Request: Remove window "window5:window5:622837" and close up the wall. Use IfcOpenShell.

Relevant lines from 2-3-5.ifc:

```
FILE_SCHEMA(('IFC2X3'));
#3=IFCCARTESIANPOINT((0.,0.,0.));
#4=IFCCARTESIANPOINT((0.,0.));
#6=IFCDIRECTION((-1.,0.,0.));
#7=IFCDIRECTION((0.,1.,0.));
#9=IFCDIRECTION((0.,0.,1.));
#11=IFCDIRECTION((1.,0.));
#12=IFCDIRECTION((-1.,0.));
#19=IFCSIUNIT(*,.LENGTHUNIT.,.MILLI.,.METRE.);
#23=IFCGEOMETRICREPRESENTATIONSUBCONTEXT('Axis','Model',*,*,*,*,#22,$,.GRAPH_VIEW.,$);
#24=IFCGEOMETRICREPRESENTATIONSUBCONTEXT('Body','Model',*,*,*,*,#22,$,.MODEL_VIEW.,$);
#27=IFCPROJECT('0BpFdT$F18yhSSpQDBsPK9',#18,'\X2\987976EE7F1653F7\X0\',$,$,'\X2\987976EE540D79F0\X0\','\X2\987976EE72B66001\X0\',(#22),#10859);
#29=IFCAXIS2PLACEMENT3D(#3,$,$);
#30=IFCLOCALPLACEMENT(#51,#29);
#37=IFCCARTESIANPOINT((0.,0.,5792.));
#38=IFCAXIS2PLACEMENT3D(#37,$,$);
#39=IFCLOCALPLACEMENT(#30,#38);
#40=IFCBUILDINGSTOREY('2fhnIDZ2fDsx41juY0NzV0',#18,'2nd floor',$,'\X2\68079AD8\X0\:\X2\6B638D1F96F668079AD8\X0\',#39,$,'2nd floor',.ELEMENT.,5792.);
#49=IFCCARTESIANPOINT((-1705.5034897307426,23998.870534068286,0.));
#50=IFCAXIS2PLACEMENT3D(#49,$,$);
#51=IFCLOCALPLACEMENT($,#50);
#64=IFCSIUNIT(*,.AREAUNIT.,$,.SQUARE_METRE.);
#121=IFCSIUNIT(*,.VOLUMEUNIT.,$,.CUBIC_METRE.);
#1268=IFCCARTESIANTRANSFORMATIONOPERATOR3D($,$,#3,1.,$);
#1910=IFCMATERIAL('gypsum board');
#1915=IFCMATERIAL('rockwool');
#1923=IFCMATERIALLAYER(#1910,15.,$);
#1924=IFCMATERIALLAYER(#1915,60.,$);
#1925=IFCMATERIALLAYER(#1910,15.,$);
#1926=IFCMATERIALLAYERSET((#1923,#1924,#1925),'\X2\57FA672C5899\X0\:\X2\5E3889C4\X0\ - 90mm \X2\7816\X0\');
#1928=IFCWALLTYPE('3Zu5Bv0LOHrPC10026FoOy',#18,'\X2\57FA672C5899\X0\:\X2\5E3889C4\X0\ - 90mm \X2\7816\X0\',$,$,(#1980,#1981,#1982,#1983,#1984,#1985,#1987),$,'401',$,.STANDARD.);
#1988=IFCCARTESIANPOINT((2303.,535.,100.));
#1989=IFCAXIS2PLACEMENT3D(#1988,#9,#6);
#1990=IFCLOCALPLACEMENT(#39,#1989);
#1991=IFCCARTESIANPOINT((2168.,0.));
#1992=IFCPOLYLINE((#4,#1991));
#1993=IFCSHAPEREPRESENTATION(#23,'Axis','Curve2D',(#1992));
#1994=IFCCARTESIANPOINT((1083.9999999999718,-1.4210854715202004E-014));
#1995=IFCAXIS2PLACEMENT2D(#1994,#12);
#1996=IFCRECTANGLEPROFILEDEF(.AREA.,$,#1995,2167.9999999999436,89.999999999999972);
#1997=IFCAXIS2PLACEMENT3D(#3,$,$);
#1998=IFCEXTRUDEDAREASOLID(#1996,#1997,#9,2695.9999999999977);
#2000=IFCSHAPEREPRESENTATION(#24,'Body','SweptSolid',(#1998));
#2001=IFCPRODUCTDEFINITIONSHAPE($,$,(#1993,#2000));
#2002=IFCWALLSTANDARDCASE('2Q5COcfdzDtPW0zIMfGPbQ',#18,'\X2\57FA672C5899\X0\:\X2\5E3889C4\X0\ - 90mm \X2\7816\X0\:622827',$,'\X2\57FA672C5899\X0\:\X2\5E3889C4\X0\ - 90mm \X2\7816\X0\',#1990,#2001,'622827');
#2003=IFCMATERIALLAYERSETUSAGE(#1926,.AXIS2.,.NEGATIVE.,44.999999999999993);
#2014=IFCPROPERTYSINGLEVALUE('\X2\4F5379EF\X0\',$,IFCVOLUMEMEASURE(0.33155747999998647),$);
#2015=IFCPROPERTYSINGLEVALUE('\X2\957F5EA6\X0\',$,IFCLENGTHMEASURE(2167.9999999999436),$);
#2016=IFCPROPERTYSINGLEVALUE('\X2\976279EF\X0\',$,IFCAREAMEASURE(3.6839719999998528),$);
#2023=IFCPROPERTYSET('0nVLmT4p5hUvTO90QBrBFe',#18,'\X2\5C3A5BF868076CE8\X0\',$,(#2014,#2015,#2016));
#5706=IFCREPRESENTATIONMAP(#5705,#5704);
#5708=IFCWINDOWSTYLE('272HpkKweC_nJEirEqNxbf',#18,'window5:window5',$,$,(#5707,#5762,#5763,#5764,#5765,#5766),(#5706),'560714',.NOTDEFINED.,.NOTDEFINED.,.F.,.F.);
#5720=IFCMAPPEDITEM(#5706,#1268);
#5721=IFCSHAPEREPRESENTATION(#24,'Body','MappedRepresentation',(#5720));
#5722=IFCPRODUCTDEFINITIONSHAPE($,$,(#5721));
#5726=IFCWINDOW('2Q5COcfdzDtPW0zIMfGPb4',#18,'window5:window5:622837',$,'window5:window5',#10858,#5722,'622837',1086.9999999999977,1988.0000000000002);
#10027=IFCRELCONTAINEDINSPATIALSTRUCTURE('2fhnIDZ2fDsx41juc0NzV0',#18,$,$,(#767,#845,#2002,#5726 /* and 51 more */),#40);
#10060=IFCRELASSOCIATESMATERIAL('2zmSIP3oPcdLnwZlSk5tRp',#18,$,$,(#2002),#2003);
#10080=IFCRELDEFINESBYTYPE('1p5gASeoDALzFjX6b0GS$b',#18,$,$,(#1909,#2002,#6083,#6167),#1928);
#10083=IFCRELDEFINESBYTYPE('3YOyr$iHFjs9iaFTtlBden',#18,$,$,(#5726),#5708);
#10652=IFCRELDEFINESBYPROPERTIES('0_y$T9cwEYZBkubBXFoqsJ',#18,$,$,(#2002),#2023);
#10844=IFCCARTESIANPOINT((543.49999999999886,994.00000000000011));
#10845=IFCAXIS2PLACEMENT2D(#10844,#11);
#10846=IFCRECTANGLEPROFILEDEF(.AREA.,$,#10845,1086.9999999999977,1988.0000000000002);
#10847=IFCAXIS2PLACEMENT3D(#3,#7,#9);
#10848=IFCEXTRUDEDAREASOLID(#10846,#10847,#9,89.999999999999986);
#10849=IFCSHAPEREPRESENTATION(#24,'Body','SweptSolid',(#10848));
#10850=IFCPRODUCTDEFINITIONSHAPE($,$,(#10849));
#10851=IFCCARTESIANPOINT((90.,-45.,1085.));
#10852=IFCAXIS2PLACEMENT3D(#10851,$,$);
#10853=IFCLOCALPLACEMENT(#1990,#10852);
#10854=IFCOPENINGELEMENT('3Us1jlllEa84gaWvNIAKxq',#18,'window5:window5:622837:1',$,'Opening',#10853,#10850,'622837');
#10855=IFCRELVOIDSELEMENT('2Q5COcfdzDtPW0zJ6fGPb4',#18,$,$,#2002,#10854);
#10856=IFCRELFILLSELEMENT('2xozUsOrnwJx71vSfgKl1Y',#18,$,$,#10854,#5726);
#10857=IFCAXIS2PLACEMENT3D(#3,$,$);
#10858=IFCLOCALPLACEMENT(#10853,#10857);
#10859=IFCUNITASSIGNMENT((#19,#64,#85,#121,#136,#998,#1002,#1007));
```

```python
import ifcopenshell
import ifcopenshell.api.feature
import ifcopenshell.api.pset
import ifcopenshell.api.root
import ifcopenshell.geom
import ifcopenshell.util.element
import ifcopenshell.util.shape
import ifcopenshell.util.unit

model = ifcopenshell.open("2-3-5.ifc")
area_scale = ifcopenshell.util.unit.calculate_unit_scale(model, "AREAUNIT")
volume_scale = ifcopenshell.util.unit.calculate_unit_scale(model, "VOLUMEUNIT")
settings = ifcopenshell.geom.settings()


def volume(element):
    """Net volume in cubic metres, openings subtracted."""
    shape = ifcopenshell.geom.create_shape(settings, element)
    return ifcopenshell.util.shape.get_volume(shape.geometry)


window = model.by_guid("2Q5COcfdzDtPW0zIMfGPb4")
opening = window.FillsVoids[0].RelatingOpeningElement
wall = opening.VoidsElements[0].RelatingBuildingElement
before = volume(wall)

ifcopenshell.api.root.remove_product(model, product=window)
ifcopenshell.api.feature.remove_feature(model, feature=opening)

after = volume(wall)
thickness = 0.09  # wall thickness in metres

# Update the wall's stored quantities.
pset = model.by_id(ifcopenshell.util.element.get_pset(wall, "尺寸标注", should_inherit=False)["id"])
ifcopenshell.api.pset.edit_pset(model, pset=pset, properties={
    "体积": model.create_entity("IfcVolumeMeasure", after / volume_scale),
    "面积": model.create_entity("IfcAreaMeasure", after / thickness / area_scale),
})

print(f"wall volume {before:.3f} -> {after:.3f} m3")

model.write("2-3-5_v2.ifc")
```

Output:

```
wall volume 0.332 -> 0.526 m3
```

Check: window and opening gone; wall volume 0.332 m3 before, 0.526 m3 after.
